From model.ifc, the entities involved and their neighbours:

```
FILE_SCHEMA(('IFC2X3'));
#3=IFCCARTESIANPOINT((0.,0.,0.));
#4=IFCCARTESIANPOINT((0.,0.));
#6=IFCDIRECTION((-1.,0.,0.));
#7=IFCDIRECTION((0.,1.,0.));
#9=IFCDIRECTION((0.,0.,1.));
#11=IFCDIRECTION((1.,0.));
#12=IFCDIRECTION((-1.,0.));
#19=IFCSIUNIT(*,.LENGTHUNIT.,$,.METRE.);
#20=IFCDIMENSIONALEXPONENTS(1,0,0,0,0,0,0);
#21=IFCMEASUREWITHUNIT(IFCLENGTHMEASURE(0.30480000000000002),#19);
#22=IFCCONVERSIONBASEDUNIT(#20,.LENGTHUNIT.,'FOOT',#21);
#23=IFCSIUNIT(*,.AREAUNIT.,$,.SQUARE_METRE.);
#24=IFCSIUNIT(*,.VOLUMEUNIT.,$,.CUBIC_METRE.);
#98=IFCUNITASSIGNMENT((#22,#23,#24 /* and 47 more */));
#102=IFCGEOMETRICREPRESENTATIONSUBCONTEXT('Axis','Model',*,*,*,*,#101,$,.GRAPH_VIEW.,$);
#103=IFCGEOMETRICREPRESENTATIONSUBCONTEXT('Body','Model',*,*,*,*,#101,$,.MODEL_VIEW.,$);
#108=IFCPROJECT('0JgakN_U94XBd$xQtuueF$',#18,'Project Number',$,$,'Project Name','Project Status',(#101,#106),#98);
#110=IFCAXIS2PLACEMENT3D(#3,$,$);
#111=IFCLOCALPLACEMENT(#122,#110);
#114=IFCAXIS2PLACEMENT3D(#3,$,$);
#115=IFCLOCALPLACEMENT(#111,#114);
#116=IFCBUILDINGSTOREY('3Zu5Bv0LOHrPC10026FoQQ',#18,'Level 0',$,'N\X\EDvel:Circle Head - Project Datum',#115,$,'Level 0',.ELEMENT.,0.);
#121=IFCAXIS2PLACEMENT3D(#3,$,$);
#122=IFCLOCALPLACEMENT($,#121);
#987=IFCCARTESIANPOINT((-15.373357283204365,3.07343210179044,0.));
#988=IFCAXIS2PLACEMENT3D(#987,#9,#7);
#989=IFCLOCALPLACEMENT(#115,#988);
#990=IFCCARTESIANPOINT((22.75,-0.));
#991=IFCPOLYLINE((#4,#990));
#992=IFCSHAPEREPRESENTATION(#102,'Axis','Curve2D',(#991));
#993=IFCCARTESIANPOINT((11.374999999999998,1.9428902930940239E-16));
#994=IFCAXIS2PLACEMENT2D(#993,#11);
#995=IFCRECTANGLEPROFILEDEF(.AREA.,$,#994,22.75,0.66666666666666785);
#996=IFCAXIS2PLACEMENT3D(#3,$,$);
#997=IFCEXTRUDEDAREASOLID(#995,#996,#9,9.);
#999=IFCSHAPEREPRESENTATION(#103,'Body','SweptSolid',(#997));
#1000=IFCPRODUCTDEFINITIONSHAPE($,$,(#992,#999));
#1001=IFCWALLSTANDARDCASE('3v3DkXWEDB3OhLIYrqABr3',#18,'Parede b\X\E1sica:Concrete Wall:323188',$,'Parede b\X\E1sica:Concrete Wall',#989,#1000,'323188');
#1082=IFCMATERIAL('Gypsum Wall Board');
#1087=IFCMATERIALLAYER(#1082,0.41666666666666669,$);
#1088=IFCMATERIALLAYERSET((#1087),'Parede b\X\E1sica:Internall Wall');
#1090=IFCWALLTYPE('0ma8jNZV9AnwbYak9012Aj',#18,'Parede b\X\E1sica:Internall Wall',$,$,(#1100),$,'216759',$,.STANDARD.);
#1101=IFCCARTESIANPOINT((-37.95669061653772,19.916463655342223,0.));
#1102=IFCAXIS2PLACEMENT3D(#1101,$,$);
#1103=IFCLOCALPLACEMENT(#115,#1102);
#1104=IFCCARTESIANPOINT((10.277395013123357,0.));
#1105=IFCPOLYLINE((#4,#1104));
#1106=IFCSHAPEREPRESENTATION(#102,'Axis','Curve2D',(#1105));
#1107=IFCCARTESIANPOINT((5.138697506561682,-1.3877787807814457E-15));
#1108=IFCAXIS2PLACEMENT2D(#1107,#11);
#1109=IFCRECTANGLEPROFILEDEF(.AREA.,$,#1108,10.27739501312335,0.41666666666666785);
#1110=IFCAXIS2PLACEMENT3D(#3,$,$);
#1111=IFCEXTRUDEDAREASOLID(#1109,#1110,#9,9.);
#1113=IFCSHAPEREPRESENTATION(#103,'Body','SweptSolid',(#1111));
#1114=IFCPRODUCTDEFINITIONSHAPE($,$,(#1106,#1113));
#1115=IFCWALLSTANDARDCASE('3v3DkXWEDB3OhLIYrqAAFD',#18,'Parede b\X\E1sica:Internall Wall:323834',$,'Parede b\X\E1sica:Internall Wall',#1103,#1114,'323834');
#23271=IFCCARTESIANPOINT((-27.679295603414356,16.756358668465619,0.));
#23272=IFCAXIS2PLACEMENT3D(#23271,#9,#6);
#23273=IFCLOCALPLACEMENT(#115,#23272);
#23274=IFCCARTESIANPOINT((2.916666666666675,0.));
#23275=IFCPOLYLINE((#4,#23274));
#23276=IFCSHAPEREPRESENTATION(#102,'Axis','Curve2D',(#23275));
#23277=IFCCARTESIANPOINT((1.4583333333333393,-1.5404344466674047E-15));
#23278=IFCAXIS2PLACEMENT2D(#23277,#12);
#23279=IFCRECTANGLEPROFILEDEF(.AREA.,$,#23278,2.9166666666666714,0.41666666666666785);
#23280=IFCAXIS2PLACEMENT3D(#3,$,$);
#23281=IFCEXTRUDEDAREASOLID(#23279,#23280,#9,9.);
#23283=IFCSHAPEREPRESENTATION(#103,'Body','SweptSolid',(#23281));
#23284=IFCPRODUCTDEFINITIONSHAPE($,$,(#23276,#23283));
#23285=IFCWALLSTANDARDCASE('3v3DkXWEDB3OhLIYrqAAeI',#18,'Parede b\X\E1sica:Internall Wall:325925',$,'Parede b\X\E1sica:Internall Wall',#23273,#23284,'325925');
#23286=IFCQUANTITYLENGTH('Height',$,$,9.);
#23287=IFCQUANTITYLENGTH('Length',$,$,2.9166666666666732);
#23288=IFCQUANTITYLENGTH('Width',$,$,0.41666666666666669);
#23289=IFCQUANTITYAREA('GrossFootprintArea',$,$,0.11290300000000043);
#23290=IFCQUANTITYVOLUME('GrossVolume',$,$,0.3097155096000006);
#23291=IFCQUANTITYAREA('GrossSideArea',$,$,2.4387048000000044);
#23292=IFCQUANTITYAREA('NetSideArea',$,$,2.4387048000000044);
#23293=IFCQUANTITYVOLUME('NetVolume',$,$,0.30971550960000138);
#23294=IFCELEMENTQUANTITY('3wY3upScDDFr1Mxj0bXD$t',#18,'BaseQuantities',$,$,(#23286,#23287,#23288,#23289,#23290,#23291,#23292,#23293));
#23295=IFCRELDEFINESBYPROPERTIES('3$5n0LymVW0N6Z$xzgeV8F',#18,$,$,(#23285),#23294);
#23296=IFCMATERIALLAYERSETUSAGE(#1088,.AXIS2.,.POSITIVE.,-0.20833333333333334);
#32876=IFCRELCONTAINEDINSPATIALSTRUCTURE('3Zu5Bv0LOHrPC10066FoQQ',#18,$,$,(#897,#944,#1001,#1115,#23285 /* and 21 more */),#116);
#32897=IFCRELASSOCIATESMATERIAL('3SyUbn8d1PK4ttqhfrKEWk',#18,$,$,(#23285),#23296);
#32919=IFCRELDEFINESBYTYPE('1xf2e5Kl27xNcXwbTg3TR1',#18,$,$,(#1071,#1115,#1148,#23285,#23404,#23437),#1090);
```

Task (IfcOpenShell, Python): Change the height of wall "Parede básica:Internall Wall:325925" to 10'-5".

```python
import ifcopenshell
import ifcopenshell.api.pset
import ifcopenshell.geom
import ifcopenshell.util.element
import ifcopenshell.util.representation
import ifcopenshell.util.shape
import ifcopenshell.util.unit

model = ifcopenshell.open("model.ifc")
unit_scale = ifcopenshell.util.unit.calculate_unit_scale(model)
area_scale = ifcopenshell.util.unit.calculate_unit_scale(model, "AREAUNIT")
volume_scale = ifcopenshell.util.unit.calculate_unit_scale(model, "VOLUMEUNIT")
settings = ifcopenshell.geom.settings()


def volume(element):
    """Net volume in cubic metres, openings subtracted."""
    shape = ifcopenshell.geom.create_shape(settings, element)
    return ifcopenshell.util.shape.get_volume(shape.geometry)


wall = model.by_guid("3v3DkXWEDB3OhLIYrqAAeI")
before = volume(wall)

body = ifcopenshell.util.representation.get_representation(wall, "Model", "Body")
solid = body.Items[0]
old_height = solid.Depth
solid.Depth = 125 * 0.0254 / unit_scale
after = volume(wall)
thickness = 0.127  # wall thickness in metres

# Update the stored height, areas and volumes.
qto = model.by_id(ifcopenshell.util.element.get_pset(wall, "BaseQuantities", should_inherit=False)["id"])
ifcopenshell.api.pset.edit_qto(model, qto=qto, properties={
    "Height": solid.Depth,
    "GrossVolume": ifcopenshell.util.element.get_pset(wall, "BaseQuantities", "GrossVolume") * solid.Depth / old_height,
    "GrossSideArea": ifcopenshell.util.element.get_pset(wall, "BaseQuantities", "GrossSideArea") * solid.Depth / old_height,
    "NetSideArea": after / thickness / area_scale,
    "NetVolume": after / volume_scale,
})

print(f"height {old_height:g} -> {solid.Depth:g}, volume {before:.3f} -> {after:.3f} m3")

model.write("model_rev.ifc")
```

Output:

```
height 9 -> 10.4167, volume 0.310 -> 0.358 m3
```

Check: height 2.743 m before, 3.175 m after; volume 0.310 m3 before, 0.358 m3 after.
